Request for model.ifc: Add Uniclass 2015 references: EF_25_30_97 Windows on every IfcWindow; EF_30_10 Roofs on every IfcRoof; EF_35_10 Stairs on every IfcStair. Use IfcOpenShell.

First a look at what the model holds.

```python
import ifcopenshell

model = ifcopenshell.open("model.ifc")
print(model.schema)
print("classifications:", [c.Name for c in model.by_type("IfcClassification")])
for ifc_class in ("IfcDoor", "IfcRoof", "IfcStair", "IfcWall", "IfcWindow"):
    print(ifc_class, len(model.by_type(ifc_class)))
```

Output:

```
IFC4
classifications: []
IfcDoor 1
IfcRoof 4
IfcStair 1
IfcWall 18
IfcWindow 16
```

```python
import ifcopenshell
import ifcopenshell.api.classification

model = ifcopenshell.open("model.ifc")

system = ifcopenshell.api.classification.add_classification(model, classification="Uniclass 2015")

codes = {
    "IfcWindow": ("EF_25_30_97", "Windows"),
    "IfcRoof": ("EF_30_10", "Roofs"),
    "IfcStair": ("EF_35_10", "Stairs"),
}
for ifc_class, (code, name) in codes.items():
    products = model.by_type(ifc_class)
    ifcopenshell.api.classification.add_reference(
        model, products=products, classification=system, identification=code, name=name
    )
    print(code, len(products))

model.write("model_edited.ifc")
```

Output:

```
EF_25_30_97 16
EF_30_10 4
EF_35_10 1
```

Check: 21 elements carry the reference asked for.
